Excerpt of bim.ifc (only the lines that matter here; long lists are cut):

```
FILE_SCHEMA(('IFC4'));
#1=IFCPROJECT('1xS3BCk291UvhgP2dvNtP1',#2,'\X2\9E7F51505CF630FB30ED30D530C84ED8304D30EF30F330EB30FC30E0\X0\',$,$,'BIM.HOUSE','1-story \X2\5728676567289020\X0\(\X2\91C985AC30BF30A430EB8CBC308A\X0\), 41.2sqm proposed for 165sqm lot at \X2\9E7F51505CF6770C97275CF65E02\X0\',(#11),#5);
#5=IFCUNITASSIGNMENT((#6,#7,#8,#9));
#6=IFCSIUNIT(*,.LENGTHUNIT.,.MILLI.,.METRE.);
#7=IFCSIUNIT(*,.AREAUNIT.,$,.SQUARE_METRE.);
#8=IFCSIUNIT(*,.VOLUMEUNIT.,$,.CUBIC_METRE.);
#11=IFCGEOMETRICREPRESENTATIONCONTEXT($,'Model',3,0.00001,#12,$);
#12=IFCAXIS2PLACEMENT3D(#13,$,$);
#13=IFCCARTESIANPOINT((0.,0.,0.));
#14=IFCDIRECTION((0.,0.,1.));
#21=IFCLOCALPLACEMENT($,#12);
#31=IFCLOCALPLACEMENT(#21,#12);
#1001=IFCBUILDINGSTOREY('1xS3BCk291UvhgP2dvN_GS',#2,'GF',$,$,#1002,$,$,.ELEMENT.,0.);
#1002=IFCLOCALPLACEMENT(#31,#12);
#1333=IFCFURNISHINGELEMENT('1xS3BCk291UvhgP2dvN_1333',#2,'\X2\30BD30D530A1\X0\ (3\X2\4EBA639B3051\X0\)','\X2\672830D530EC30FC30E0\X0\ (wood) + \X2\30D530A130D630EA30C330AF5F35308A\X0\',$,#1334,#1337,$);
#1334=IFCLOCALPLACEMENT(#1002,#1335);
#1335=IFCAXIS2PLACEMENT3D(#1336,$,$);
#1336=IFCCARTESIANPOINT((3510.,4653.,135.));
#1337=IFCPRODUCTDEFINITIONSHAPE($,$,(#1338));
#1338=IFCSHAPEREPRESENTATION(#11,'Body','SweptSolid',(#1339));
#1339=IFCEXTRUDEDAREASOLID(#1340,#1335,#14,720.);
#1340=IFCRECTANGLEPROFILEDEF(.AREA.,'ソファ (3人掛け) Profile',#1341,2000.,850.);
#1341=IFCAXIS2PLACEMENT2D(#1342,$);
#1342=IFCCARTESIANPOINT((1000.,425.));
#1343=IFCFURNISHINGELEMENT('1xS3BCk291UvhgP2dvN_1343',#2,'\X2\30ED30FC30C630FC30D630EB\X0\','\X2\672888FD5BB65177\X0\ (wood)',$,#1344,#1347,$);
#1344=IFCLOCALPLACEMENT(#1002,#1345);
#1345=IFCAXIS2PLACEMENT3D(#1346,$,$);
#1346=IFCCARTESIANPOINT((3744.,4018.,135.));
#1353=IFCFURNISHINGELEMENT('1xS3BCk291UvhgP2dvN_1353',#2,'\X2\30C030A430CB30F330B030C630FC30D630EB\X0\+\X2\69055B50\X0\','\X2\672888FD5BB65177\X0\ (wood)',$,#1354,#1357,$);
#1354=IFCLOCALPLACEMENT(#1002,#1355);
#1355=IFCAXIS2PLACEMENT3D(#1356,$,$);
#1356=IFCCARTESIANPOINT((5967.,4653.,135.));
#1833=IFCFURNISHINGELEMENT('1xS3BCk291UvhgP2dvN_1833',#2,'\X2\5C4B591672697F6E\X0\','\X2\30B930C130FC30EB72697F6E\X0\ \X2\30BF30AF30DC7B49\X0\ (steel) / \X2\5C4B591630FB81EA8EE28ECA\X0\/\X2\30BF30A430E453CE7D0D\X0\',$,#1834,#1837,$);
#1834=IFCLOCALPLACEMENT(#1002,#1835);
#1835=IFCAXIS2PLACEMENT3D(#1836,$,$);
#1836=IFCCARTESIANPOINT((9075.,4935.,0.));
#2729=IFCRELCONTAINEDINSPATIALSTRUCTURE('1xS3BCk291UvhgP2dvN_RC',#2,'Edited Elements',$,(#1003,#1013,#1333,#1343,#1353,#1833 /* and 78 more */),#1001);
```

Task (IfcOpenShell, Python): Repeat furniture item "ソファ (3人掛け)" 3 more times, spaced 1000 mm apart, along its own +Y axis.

```python
import ifcopenshell
import ifcopenshell.api.geometry
import ifcopenshell.api.root
import ifcopenshell.util.element
import ifcopenshell.util.placement

model = ifcopenshell.open("bim.ifc")


def reuse_history(source, copy):
    """copy_class also copies each property set's owner history, people and application; keep the originals."""
    for rel in copy.IsDefinedBy:
        if rel.is_a("IfcRelDefinesByProperties") and (history := rel.RelatingPropertyDefinition.OwnerHistory):
            rel.RelatingPropertyDefinition.OwnerHistory = source.OwnerHistory
            ifcopenshell.util.element.remove_deep2(model, history)


source = model.by_guid("1xS3BCk291UvhgP2dvN_1333")
base = ifcopenshell.util.placement.get_local_placement(source.ObjectPlacement)
step = base[:3, 1] * 1000.0

for i in range(1, 4):
    copy = ifcopenshell.api.root.copy_class(model, product=source)
    copy.Representation = ifcopenshell.util.element.copy_deep(
        model, source.Representation, exclude=["IfcGeometricRepresentationContext", "IfcRepresentationMap"]
    )
    reuse_history(source, copy)
    matrix = base.copy()
    matrix[:3, 3] += i * step
    print("added at", matrix[:3, 3].round(3) + 0.0)
    ifcopenshell.api.geometry.edit_object_placement(model, product=copy, matrix=matrix, is_si=False)

model.write("bim_updated.ifc")
```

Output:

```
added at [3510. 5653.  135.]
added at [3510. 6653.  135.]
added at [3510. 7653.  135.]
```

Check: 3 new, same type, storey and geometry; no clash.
